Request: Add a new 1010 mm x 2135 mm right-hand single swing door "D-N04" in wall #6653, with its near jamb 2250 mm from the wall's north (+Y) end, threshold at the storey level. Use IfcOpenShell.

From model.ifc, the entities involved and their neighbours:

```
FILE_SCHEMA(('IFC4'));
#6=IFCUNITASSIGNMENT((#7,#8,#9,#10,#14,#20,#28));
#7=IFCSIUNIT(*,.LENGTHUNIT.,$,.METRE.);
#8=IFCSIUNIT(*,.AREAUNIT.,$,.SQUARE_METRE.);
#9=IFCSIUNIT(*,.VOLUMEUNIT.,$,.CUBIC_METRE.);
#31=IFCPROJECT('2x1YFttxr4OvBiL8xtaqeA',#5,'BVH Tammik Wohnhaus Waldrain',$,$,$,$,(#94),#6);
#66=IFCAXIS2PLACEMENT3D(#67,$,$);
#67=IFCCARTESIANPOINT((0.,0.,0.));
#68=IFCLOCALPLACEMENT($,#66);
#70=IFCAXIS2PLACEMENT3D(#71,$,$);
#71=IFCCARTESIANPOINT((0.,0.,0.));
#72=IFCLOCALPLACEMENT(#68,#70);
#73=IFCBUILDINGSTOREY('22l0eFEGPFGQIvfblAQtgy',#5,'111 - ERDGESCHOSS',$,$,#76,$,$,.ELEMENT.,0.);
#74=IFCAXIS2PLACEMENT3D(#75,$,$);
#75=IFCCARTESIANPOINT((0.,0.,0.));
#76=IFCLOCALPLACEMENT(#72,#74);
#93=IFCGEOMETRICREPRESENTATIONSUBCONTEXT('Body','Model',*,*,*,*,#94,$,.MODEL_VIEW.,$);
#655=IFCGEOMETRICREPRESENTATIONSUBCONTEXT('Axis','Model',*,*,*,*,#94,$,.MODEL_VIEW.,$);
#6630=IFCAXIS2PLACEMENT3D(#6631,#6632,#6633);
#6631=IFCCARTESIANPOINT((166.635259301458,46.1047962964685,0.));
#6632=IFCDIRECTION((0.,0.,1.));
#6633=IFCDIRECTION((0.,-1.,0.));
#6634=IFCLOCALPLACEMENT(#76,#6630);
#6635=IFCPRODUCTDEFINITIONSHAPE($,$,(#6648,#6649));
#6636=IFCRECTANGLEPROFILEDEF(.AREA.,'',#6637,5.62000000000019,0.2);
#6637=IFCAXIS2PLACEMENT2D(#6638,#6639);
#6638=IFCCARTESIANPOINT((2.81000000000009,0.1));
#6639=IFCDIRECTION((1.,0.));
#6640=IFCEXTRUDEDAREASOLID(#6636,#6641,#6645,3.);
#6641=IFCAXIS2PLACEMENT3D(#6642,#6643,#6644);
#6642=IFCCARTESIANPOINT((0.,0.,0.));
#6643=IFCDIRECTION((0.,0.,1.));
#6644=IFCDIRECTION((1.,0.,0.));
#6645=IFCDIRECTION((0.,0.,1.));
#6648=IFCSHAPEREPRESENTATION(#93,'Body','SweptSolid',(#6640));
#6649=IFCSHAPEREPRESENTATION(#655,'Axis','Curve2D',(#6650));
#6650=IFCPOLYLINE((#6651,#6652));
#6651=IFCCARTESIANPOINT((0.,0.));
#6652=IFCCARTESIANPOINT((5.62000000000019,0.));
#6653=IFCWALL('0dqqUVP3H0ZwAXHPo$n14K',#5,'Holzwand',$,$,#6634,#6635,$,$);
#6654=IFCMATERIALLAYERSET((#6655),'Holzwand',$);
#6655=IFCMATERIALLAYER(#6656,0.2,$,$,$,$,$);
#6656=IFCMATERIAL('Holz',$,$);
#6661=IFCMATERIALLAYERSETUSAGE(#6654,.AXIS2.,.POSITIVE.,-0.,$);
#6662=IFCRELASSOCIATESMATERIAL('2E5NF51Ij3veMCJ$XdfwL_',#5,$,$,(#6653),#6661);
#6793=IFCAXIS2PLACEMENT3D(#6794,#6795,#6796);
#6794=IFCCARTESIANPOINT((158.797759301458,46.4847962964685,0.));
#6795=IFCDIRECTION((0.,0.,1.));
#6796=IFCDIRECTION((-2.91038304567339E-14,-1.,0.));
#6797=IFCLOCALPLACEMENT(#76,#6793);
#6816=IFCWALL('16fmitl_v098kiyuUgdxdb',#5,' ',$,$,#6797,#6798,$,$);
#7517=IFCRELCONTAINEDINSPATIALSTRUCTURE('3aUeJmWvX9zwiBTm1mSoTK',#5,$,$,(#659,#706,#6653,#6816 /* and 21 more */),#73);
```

```python
import numpy as np
import ifcopenshell
import ifcopenshell.api.feature
import ifcopenshell.api.geometry
import ifcopenshell.api.root
import ifcopenshell.api.spatial
import ifcopenshell.geom
import ifcopenshell.util.element
import ifcopenshell.util.placement
import ifcopenshell.util.representation
import ifcopenshell.util.shape
import ifcopenshell.util.unit

model = ifcopenshell.open("model.ifc")
unit_scale = ifcopenshell.util.unit.calculate_unit_scale(model)
settings = ifcopenshell.geom.settings()


def volume(element):
    """Net volume in cubic metres, openings subtracted."""
    shape = ifcopenshell.geom.create_shape(settings, element)
    return ifcopenshell.util.shape.get_volume(shape.geometry)


wall = model.by_guid("0dqqUVP3H0ZwAXHPo$n14K")
storey = ifcopenshell.util.element.get_container(wall, ifc_class="IfcBuildingStorey")
context = ifcopenshell.util.representation.get_context(model, "Model", "Body", "MODEL_VIEW")
before = volume(wall)

width, height, from_end, sill = 1.01, 2.135, 2.25, 0.0  # metres

# The wall runs along its own X axis, and the end named is its -X end.
wall_shape = ifcopenshell.geom.create_shape(settings, wall)
x, y, z = ifcopenshell.util.shape.get_vertices(wall_shape.geometry).T
start = x.min() + from_end
face, thickness = float(y.min()), float(y.max() - y.min())
wall_matrix = ifcopenshell.util.placement.get_local_placement(wall.ObjectPlacement)
level = ifcopenshell.util.placement.get_local_placement(storey.ObjectPlacement)[2, 3]


def in_wall(x, y):
    """Placement at x, y metres in the wall's axes, at sill height."""
    matrix = wall_matrix.copy()
    matrix[:, 3] = wall_matrix @ np.array([x / unit_scale, y / unit_scale, 0.0, 1.0])
    matrix[2, 3] = level + sill / unit_scale
    return matrix


# Opening: a box that overshoots both wall faces by 50 mm.
opening = ifcopenshell.api.root.create_entity(model, ifc_class="IfcOpeningElement", predefined_type="OPENING")
box = ifcopenshell.api.geometry.add_wall_representation(
    model, context=context, length=width, height=height, thickness=thickness + 0.1
)
ifcopenshell.api.geometry.assign_representation(model, product=opening, representation=box)
ifcopenshell.api.geometry.edit_object_placement(model, product=opening, matrix=in_wall(start, face - 0.05), is_si=False)
ifcopenshell.api.feature.add_feature(model, feature=opening, element=wall)

door = ifcopenshell.api.root.create_entity(model, ifc_class="IfcDoor", name="D-N04", predefined_type="DOOR")
door.OverallWidth, door.OverallHeight = width / unit_scale, height / unit_scale
door.OperationType = "SINGLE_SWING_RIGHT"
body = ifcopenshell.api.geometry.add_door_representation(
    model,
    context=context,
    overall_width=door.OverallWidth,
    overall_height=door.OverallHeight,
    operation_type="SINGLE_SWING_RIGHT",
    lining_properties={"LiningDepth": thickness / unit_scale, "ThresholdDepth": thickness / unit_scale},
)
ifcopenshell.api.geometry.assign_representation(model, product=door, representation=body)
ifcopenshell.api.spatial.assign_container(model, products=[door], relating_structure=storey)
ifcopenshell.api.feature.add_filling(model, opening=opening, element=door)

# The lining spans the wall, so the door starts at the wall face.
ifcopenshell.api.geometry.edit_object_placement(model, product=door, matrix=in_wall(start, face), is_si=False)

after = volume(wall)

print(f"wall volume {before:.3f} -> {after:.3f} m3")

model.write("model_v2.ifc")
```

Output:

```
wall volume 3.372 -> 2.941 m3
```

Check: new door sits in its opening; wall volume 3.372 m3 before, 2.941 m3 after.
